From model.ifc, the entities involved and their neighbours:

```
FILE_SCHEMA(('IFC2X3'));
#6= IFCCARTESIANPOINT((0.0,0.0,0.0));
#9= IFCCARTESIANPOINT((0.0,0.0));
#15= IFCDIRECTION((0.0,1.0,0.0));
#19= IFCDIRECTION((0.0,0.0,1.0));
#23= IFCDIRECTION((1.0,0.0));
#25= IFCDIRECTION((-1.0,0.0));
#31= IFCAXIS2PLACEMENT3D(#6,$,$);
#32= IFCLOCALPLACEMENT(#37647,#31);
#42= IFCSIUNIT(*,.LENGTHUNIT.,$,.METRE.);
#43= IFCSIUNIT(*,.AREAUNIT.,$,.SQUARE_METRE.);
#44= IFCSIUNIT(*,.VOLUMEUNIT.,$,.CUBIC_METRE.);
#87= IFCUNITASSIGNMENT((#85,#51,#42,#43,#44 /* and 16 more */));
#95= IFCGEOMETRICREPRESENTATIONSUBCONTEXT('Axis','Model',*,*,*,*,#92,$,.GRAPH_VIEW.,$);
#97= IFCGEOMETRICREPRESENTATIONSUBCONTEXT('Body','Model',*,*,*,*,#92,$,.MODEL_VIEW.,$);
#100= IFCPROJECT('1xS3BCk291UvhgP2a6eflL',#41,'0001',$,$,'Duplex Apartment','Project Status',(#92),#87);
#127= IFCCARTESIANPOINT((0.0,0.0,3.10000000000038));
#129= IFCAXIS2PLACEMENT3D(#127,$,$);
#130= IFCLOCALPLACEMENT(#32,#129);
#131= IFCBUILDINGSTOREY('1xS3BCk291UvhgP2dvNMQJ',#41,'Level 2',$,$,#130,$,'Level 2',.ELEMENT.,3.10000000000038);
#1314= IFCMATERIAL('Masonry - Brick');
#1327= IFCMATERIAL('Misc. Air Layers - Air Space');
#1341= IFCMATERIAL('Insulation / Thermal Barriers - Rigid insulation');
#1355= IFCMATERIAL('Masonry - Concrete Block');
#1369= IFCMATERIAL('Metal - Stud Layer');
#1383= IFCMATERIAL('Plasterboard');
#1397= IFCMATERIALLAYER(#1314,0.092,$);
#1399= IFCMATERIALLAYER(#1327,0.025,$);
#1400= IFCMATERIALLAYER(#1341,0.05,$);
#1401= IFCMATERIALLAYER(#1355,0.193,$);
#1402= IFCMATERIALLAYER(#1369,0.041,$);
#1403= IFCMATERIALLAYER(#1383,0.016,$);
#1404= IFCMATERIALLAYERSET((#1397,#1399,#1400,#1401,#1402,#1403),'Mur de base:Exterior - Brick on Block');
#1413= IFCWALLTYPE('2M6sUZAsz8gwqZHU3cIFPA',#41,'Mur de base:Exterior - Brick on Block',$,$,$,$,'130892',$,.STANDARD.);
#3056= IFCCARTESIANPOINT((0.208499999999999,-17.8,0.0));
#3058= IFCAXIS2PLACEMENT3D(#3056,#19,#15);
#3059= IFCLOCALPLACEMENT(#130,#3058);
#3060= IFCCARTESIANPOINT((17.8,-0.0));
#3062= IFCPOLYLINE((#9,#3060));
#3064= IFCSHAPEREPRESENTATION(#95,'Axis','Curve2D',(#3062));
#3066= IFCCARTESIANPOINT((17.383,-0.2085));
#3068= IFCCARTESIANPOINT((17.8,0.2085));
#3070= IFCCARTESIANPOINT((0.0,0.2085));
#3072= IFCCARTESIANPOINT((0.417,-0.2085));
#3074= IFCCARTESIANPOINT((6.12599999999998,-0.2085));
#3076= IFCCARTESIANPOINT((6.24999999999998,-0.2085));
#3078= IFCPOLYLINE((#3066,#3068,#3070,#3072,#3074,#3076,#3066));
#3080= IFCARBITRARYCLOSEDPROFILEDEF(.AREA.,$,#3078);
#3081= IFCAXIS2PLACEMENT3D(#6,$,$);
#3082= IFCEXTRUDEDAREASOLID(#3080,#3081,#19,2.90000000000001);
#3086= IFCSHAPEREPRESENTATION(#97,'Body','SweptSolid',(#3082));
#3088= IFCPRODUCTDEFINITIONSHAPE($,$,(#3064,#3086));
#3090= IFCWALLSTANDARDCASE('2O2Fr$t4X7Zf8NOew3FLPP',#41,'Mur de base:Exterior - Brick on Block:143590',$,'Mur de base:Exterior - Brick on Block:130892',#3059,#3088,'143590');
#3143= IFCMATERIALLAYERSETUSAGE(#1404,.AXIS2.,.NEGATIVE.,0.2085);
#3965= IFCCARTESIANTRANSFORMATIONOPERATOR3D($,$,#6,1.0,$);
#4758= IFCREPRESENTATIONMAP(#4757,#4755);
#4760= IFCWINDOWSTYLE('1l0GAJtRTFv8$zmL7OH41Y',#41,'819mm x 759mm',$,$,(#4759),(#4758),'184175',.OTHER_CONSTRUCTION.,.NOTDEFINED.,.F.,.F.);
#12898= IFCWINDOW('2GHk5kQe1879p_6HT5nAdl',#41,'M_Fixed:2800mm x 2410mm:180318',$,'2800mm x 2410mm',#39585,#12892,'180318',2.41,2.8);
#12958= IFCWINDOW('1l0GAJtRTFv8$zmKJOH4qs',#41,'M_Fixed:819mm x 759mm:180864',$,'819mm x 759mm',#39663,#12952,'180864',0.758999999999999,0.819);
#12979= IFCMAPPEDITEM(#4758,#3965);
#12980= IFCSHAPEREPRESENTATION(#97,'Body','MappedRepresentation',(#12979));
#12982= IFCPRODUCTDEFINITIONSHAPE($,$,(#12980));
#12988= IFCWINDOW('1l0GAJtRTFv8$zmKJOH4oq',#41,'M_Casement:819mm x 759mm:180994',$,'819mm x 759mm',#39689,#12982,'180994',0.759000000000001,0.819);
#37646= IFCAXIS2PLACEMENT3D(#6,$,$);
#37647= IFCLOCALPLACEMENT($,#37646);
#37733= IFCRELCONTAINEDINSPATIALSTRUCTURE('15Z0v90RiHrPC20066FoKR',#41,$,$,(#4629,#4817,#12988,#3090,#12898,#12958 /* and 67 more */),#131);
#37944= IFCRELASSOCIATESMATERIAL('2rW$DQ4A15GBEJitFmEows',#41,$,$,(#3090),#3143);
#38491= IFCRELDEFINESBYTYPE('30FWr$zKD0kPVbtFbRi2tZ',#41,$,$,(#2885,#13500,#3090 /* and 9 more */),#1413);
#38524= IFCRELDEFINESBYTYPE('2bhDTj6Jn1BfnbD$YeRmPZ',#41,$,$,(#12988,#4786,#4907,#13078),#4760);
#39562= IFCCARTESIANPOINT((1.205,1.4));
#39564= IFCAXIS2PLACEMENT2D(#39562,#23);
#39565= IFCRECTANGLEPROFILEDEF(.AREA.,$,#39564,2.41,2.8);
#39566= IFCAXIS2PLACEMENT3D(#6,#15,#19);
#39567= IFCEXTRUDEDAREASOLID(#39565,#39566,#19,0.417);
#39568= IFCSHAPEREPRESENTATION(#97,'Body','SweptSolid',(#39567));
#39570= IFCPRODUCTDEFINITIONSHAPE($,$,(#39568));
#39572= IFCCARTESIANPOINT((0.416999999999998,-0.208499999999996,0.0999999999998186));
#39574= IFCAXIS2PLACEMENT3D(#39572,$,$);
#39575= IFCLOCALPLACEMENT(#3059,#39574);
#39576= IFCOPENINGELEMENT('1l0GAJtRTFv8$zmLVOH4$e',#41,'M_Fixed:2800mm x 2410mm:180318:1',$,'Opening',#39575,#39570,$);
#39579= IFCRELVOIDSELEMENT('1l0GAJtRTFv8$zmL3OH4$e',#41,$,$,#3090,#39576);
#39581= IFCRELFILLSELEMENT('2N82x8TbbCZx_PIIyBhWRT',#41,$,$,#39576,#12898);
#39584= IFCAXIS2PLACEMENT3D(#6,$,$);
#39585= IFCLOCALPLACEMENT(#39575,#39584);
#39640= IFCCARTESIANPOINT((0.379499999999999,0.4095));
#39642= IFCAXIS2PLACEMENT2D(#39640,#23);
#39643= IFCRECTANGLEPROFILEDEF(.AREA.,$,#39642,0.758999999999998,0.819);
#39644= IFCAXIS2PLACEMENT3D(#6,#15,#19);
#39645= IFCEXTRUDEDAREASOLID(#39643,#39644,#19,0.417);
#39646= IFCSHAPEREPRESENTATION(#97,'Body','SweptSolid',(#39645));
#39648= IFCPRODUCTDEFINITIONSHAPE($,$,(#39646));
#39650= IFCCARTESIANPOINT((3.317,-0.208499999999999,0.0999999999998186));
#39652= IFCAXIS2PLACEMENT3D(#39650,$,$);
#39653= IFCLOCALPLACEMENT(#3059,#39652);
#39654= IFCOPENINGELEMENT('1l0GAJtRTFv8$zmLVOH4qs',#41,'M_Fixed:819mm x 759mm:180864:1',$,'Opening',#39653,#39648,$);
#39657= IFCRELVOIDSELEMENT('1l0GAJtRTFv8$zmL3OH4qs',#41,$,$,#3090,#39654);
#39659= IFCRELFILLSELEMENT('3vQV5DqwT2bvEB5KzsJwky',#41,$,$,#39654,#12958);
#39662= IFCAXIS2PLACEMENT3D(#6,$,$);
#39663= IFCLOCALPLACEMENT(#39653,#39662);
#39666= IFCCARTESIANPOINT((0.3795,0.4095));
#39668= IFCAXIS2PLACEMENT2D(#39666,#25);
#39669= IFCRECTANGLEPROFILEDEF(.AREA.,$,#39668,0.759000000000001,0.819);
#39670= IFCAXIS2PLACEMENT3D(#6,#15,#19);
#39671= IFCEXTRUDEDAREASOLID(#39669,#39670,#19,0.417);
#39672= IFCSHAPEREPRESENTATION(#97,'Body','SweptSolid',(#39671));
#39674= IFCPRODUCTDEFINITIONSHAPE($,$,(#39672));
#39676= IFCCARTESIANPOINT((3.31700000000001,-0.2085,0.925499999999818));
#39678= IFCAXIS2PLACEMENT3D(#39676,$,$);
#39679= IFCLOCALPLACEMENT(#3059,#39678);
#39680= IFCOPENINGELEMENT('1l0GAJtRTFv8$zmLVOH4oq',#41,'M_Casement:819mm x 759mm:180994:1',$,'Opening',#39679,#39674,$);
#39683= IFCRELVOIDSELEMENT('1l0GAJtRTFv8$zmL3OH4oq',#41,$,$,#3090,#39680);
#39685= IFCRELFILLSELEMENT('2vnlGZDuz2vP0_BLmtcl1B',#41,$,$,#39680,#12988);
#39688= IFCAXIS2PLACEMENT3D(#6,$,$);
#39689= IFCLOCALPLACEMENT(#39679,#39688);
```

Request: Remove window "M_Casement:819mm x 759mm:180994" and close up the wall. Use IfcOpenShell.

```python
import ifcopenshell
import ifcopenshell.api.feature
import ifcopenshell.api.root
import ifcopenshell.geom
import ifcopenshell.util.shape

model = ifcopenshell.open("model.ifc")
settings = ifcopenshell.geom.settings()


def volume(element):
    """Net volume in cubic metres, openings subtracted."""
    shape = ifcopenshell.geom.create_shape(settings, element)
    return ifcopenshell.util.shape.get_volume(shape.geometry)


window = model.by_id(12988)
opening = window.FillsVoids[0].RelatingOpeningElement
wall = opening.VoidsElements[0].RelatingBuildingElement
before = volume(wall)

ifcopenshell.api.root.remove_product(model, product=window)
ifcopenshell.api.feature.remove_feature(model, feature=opening)

after = volume(wall)

print(f"wall volume {before:.3f} -> {after:.3f} m3")

model.write("model_v2.ifc")
```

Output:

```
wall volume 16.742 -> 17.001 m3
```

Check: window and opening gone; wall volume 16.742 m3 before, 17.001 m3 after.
